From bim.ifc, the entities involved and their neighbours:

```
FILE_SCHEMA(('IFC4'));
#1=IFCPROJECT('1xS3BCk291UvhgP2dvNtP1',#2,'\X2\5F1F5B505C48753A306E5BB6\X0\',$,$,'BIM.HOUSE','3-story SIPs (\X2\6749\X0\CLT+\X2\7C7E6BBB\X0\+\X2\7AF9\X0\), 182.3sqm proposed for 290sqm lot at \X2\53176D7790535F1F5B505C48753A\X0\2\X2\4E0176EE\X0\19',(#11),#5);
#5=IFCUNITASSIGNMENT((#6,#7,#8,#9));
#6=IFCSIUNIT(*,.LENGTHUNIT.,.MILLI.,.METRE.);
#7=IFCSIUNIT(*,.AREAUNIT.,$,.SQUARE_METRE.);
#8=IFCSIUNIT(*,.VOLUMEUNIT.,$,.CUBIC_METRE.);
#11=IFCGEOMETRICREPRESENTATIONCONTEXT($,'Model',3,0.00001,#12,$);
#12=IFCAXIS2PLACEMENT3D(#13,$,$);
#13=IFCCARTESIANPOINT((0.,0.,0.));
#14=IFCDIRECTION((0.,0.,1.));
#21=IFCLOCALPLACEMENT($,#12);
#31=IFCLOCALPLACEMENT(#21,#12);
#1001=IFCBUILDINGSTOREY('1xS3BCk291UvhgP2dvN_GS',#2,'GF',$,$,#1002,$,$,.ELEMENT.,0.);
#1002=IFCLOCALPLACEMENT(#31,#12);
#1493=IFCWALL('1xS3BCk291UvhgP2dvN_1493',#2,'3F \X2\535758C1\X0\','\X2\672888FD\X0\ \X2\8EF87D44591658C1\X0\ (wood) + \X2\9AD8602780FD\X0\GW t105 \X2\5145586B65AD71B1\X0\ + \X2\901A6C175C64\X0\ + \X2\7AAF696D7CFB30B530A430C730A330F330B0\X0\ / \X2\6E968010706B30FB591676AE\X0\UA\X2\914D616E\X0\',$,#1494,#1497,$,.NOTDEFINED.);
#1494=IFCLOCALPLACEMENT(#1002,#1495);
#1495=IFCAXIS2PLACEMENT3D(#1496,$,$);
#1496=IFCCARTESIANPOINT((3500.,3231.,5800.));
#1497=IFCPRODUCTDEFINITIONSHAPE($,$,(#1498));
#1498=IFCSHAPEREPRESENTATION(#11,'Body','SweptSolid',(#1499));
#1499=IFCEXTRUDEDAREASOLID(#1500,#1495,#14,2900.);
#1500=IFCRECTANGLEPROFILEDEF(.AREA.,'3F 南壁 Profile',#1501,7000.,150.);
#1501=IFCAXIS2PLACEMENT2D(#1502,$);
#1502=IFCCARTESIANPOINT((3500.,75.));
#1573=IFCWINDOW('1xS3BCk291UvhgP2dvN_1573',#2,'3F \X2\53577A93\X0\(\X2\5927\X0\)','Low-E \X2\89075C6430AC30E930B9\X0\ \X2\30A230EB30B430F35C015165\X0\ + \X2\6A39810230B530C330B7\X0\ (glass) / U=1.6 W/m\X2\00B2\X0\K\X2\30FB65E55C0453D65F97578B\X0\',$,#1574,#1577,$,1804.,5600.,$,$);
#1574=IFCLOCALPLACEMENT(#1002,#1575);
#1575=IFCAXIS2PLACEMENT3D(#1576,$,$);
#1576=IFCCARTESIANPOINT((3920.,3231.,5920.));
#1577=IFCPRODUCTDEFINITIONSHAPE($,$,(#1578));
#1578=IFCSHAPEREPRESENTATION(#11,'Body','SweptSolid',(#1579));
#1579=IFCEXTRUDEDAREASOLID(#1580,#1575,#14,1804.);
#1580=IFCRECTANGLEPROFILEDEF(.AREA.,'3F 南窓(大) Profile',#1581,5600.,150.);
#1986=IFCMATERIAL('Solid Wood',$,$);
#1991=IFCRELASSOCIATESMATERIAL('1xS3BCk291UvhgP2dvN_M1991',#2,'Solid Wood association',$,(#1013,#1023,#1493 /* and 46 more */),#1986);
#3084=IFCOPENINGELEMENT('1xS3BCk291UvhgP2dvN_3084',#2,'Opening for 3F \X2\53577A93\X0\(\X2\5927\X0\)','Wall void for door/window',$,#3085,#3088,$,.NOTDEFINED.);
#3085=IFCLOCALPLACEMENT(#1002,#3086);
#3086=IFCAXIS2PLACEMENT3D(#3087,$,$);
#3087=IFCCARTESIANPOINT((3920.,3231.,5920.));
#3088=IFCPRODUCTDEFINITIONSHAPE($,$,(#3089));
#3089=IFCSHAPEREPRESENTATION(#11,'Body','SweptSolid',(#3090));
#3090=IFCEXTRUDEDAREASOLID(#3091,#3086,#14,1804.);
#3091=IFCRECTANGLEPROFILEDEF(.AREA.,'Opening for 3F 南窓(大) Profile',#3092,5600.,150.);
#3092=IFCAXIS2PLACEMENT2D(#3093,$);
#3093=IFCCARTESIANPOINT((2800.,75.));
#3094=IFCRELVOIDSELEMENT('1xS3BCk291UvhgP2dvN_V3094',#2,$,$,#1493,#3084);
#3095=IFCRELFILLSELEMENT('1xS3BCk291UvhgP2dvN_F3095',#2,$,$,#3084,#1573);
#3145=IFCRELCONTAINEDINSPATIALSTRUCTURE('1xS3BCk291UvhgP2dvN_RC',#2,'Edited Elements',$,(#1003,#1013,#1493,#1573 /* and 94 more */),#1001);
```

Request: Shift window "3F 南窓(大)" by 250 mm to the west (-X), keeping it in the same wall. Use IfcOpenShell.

```python
import ifcopenshell
import ifcopenshell.api.geometry
import ifcopenshell.util.placement
import ifcopenshell.util.unit

model = ifcopenshell.open("bim.ifc")
unit_scale = ifcopenshell.util.unit.calculate_unit_scale(model)

window = model.by_id(1573)
opening = window.FillsVoids[0].RelatingOpeningElement
wall = opening.VoidsElements[0].RelatingBuildingElement

wall_matrix = ifcopenshell.util.placement.get_local_placement(wall.ObjectPlacement)
shift = wall_matrix[:3, 0] * -0.25 / unit_scale
before = ifcopenshell.util.placement.get_local_placement(window.ObjectPlacement)[:3, 3].copy()

# The window is not placed relative to its opening, so move both.
for product in (opening, window):
    matrix = ifcopenshell.util.placement.get_local_placement(product.ObjectPlacement)
    matrix[:3, 3] += shift
    ifcopenshell.api.geometry.edit_object_placement(model, product=product, matrix=matrix, is_si=False)

after = ifcopenshell.util.placement.get_local_placement(window.ObjectPlacement)[:3, 3]
print("window moved by", (after - before).round(3) + 0.0)

model.write("bim_edited.ifc")
```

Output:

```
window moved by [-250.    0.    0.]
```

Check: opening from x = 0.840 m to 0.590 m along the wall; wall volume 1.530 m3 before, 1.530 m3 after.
